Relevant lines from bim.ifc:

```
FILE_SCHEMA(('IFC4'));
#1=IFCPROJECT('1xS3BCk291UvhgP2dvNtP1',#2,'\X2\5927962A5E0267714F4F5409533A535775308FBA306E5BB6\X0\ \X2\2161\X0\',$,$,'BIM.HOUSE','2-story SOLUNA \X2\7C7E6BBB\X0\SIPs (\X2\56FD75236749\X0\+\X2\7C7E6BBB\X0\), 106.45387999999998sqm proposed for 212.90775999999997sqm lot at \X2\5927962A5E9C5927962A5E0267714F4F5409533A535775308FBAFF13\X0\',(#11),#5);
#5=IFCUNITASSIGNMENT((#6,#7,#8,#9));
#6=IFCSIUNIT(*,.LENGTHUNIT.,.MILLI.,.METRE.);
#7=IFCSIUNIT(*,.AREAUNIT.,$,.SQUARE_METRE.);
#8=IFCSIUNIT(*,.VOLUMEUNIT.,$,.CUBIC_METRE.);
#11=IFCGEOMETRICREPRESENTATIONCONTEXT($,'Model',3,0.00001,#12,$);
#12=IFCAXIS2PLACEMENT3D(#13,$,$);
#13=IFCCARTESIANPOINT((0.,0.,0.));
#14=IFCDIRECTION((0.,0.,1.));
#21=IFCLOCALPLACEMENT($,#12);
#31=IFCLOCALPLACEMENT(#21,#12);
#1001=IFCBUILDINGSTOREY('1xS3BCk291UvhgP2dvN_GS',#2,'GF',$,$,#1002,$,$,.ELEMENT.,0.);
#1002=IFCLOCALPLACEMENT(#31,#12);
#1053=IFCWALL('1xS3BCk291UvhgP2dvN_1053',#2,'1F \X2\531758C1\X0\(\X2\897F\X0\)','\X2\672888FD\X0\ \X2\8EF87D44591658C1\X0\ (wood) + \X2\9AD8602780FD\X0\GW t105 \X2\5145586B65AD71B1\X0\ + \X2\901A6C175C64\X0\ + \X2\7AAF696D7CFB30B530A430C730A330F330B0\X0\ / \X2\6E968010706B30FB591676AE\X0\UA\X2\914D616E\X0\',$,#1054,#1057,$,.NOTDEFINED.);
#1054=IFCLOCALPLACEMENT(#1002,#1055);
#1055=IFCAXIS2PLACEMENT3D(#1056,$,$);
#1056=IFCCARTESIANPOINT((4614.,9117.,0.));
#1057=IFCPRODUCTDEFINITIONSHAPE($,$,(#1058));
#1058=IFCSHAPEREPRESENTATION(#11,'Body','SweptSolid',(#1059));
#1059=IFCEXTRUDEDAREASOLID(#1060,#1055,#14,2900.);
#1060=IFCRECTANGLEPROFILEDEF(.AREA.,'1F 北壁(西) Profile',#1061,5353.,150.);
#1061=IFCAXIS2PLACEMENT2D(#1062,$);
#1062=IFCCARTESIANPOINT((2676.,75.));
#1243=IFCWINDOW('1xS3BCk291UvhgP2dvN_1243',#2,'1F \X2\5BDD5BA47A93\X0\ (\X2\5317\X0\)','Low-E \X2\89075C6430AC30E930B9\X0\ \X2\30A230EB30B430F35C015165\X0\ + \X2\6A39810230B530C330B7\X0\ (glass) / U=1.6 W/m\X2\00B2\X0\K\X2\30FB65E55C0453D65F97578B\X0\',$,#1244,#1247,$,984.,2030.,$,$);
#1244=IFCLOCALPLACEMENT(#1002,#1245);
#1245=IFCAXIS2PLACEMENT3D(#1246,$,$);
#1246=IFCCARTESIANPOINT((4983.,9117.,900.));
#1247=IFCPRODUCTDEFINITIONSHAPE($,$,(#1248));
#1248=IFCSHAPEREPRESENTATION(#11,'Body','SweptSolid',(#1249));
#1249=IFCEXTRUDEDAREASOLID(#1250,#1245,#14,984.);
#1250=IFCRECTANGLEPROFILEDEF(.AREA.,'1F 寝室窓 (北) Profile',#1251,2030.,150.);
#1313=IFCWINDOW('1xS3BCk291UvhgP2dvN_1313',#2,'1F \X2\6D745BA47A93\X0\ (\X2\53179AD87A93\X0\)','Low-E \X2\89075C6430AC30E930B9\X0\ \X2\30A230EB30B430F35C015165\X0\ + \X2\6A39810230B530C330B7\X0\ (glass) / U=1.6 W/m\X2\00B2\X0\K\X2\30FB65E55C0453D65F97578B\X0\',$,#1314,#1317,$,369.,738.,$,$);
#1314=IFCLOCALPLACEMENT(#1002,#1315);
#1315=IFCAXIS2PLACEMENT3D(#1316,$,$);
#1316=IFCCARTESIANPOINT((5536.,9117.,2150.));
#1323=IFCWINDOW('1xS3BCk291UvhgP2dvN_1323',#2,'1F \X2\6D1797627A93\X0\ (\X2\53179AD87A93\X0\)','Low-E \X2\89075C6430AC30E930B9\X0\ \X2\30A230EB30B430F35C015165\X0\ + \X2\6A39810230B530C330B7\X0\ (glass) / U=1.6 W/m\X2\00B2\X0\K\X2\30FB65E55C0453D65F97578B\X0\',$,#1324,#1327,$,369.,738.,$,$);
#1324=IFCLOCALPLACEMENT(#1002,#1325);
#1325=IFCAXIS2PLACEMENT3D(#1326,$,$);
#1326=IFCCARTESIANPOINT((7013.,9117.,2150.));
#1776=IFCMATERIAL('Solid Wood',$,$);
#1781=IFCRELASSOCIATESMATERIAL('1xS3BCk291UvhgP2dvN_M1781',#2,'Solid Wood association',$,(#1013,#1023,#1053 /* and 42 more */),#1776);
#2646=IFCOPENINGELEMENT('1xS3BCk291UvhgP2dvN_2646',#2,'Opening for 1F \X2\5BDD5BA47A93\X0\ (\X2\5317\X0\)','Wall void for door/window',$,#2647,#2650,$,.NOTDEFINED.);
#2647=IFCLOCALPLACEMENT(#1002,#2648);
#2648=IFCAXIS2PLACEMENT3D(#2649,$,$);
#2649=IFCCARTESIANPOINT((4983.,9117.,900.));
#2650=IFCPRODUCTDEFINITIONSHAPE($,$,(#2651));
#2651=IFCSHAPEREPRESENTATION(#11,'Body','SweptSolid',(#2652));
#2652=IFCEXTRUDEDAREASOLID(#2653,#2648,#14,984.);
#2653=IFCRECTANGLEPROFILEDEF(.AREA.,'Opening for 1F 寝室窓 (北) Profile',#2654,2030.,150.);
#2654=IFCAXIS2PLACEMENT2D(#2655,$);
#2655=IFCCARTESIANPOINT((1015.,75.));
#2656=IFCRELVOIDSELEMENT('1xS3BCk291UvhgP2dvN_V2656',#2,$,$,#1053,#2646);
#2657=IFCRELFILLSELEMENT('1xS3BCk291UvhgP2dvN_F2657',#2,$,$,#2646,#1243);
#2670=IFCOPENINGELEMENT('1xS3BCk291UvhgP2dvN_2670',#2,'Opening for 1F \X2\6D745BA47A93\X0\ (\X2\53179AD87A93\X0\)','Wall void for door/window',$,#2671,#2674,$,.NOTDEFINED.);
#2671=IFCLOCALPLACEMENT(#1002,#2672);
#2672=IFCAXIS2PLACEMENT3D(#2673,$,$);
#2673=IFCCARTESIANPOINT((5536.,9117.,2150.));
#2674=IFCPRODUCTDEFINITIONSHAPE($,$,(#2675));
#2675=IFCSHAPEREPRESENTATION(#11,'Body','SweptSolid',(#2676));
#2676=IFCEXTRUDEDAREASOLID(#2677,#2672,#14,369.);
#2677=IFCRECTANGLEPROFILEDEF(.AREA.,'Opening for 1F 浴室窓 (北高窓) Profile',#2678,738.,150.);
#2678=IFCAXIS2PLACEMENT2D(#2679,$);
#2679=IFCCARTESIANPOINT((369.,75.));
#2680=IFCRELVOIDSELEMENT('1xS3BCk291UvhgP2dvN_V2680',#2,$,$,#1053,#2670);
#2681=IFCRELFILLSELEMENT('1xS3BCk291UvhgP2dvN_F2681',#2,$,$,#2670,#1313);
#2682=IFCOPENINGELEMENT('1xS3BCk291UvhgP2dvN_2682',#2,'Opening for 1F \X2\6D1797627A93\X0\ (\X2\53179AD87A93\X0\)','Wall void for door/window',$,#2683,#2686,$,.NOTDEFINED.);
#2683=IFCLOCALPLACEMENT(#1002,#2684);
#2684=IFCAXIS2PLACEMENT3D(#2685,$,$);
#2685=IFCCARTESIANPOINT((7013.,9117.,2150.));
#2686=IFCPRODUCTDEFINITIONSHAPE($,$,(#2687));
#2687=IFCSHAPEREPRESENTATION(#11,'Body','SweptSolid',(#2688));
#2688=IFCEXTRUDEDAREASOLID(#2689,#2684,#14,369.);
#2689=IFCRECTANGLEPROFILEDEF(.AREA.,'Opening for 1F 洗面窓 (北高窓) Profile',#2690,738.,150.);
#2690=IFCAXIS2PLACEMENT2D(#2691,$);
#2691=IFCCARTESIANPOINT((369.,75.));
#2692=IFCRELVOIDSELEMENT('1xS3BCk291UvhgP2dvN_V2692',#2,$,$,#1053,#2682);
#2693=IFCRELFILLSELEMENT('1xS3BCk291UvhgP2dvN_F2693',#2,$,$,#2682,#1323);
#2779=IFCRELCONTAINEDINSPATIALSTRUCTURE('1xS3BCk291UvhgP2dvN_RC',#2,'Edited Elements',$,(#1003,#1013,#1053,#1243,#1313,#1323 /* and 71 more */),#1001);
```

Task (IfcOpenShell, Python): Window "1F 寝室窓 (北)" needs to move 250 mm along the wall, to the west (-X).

```python
import ifcopenshell
import ifcopenshell.api.geometry
import ifcopenshell.util.placement
import ifcopenshell.util.unit

model = ifcopenshell.open("bim.ifc")
unit_scale = ifcopenshell.util.unit.calculate_unit_scale(model)

window = model.by_guid("1xS3BCk291UvhgP2dvN_1243")
opening = window.FillsVoids[0].RelatingOpeningElement
wall = opening.VoidsElements[0].RelatingBuildingElement

wall_matrix = ifcopenshell.util.placement.get_local_placement(wall.ObjectPlacement)
shift = wall_matrix[:3, 0] * -0.25 / unit_scale
before = ifcopenshell.util.placement.get_local_placement(window.ObjectPlacement)[:3, 3].copy()

# The window is not placed relative to its opening, so move both.
for product in (opening, window):
    matrix = ifcopenshell.util.placement.get_local_placement(product.ObjectPlacement)
    matrix[:3, 3] += shift
    ifcopenshell.api.geometry.edit_object_placement(model, product=product, matrix=matrix, is_si=False)

after = ifcopenshell.util.placement.get_local_placement(window.ObjectPlacement)[:3, 3]
print("window moved by", (after - before).round(3) + 0.0)

model.write("bim_rev.ifc")
```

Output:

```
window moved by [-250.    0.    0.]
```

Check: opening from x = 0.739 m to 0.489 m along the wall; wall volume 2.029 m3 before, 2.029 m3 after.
